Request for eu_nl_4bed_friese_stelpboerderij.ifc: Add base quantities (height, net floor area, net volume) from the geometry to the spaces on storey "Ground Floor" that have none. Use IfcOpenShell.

First a look at what the model holds.

```python
import ifcopenshell
import ifcopenshell.util.element
import ifcopenshell.util.unit

model = ifcopenshell.open("eu_nl_4bed_friese_stelpboerderij.ifc")
print(model.schema)
for unit_type in ("LENGTHUNIT", "AREAUNIT", "VOLUMEUNIT"):
    print(unit_type, ifcopenshell.util.unit.calculate_unit_scale(model, unit_type))
storey = next(s for s in model.by_type("IfcBuildingStorey") if s.Name == "Ground Floor")
spaces = [e for e in ifcopenshell.util.element.get_decomposition(storey) if e.is_a("IfcSpace")]
for e in sorted(spaces, key=lambda e: e.id()):
    print(e.id(), e.is_a(), e.Name, list(ifcopenshell.util.element.get_psets(e, qtos_only=True)), sep=" | ")
```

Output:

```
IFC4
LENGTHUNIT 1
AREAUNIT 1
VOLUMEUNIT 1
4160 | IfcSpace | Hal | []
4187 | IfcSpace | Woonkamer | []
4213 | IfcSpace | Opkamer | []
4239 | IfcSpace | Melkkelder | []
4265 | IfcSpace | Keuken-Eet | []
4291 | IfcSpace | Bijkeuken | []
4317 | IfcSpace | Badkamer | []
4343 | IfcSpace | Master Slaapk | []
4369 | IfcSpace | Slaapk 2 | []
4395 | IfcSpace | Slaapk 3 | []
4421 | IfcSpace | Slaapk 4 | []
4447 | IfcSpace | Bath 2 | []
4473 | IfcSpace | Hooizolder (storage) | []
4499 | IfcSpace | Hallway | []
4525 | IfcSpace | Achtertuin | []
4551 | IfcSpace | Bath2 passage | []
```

```python
import ifcopenshell
import ifcopenshell.api.pset
import ifcopenshell.geom
import ifcopenshell.util.element
import ifcopenshell.util.shape
import ifcopenshell.util.unit

model = ifcopenshell.open("eu_nl_4bed_friese_stelpboerderij.ifc")
unit_scale = ifcopenshell.util.unit.calculate_unit_scale(model)
area_scale = ifcopenshell.util.unit.calculate_unit_scale(model, "AREAUNIT")
volume_scale = ifcopenshell.util.unit.calculate_unit_scale(model, "VOLUMEUNIT")
settings = ifcopenshell.geom.settings()

storey = next(s for s in model.by_type("IfcBuildingStorey") if s.Name == "Ground Floor")
spaces = [e for e in ifcopenshell.util.element.get_decomposition(storey) if e.is_a("IfcSpace")]

for e in sorted(spaces, key=lambda e: e.id()):
    if ifcopenshell.util.element.get_psets(e, qtos_only=True, should_inherit=False):
        continue
    # Geometry comes back in metres, in the element's own axes.
    shape = ifcopenshell.geom.create_shape(settings, e)
    values = {
        "Height": ifcopenshell.util.shape.get_z(shape.geometry) / unit_scale,
        "NetFloorArea": ifcopenshell.util.shape.get_footprint_area(shape.geometry) / area_scale,
        "NetVolume": ifcopenshell.util.shape.get_volume(shape.geometry) / volume_scale,
    }
    qto = ifcopenshell.api.pset.add_qto(model, product=e, name="Qto_SpaceBaseQuantities")
    ifcopenshell.api.pset.edit_qto(model, qto=qto, properties=values)
    print(e.id(), {k: round(v, 3) for k, v in values.items()})

model.write("eu_nl_4bed_friese_stelpboerderij-out.ifc")
```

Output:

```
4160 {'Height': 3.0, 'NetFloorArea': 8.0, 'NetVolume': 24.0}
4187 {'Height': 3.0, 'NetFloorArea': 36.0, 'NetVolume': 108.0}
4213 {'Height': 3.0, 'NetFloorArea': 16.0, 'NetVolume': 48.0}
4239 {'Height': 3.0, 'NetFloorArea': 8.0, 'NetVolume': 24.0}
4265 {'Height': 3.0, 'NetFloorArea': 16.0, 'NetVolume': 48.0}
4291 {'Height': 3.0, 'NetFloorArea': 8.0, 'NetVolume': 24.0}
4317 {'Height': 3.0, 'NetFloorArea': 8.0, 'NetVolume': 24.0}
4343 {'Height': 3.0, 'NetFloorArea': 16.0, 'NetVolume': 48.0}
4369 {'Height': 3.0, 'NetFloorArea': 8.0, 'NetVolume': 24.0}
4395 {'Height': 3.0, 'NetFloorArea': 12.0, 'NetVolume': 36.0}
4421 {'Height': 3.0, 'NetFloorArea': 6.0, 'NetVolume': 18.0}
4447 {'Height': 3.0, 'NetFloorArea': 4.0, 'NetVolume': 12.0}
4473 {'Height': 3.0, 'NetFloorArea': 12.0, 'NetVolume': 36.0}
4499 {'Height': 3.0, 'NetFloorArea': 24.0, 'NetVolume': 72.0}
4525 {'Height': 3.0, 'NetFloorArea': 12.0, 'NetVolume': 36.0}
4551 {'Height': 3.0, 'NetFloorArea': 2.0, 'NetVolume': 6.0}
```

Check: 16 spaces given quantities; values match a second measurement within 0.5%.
